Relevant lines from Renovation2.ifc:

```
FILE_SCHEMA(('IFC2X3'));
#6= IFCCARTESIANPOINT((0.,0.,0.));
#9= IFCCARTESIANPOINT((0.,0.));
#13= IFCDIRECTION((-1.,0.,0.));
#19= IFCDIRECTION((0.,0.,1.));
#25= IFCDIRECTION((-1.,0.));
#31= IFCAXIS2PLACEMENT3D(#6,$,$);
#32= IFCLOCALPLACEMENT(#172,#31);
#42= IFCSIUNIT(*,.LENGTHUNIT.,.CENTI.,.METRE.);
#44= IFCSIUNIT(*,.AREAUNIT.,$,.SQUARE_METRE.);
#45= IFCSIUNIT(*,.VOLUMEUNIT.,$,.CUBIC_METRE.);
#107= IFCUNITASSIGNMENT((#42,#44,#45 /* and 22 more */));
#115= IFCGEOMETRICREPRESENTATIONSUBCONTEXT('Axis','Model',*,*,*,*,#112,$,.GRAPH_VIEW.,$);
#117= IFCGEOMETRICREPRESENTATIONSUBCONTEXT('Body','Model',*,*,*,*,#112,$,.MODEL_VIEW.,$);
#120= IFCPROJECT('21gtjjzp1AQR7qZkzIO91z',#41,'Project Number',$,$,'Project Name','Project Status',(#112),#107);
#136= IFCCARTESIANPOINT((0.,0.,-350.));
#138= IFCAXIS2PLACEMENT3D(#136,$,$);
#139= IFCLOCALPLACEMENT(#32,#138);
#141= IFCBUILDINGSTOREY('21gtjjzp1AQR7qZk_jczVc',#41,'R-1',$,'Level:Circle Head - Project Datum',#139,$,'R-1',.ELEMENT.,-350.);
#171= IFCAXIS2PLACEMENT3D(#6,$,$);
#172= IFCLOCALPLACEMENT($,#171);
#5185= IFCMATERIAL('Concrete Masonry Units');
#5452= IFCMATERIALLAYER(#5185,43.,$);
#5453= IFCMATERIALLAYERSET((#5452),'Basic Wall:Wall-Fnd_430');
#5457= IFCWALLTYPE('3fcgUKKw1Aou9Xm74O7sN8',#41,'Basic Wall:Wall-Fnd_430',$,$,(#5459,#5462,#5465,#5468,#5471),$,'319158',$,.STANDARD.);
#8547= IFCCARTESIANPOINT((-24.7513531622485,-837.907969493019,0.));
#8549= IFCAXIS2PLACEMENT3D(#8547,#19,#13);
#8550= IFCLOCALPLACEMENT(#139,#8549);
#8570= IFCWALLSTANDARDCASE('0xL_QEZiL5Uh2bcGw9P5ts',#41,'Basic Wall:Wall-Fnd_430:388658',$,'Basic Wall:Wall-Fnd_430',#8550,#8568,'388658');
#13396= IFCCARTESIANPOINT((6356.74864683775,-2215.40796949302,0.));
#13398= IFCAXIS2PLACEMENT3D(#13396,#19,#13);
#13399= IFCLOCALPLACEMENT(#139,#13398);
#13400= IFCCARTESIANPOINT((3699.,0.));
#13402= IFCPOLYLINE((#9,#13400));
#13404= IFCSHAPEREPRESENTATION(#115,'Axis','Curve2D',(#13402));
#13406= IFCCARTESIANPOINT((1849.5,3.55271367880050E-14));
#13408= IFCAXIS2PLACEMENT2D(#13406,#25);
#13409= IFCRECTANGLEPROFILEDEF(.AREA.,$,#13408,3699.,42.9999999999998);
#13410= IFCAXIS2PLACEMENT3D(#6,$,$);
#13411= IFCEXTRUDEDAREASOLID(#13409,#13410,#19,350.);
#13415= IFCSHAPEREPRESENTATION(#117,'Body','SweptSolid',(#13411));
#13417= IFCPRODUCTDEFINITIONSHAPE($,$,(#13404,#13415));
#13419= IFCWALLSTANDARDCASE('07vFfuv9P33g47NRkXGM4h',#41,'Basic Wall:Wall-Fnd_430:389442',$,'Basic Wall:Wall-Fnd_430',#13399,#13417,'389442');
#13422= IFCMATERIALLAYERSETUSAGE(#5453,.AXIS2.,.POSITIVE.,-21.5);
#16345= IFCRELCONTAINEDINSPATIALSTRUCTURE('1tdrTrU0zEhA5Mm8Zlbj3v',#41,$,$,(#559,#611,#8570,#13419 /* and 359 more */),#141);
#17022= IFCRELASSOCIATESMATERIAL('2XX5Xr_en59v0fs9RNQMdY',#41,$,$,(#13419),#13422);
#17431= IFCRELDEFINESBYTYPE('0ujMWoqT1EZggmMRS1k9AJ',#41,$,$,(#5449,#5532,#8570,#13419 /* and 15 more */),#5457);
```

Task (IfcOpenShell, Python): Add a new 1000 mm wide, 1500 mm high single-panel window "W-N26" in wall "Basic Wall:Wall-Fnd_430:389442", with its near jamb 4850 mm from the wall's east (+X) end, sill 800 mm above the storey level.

```python
import numpy as np
import ifcopenshell
import ifcopenshell.api.feature
import ifcopenshell.api.geometry
import ifcopenshell.api.root
import ifcopenshell.api.spatial
import ifcopenshell.api.type
import ifcopenshell.geom
import ifcopenshell.util.element
import ifcopenshell.util.placement
import ifcopenshell.util.representation
import ifcopenshell.util.shape
import ifcopenshell.util.unit

model = ifcopenshell.open("Renovation2.ifc")
unit_scale = ifcopenshell.util.unit.calculate_unit_scale(model)
settings = ifcopenshell.geom.settings()


def volume(element):
    """Net volume in cubic metres, openings subtracted."""
    shape = ifcopenshell.geom.create_shape(settings, element)
    return ifcopenshell.util.shape.get_volume(shape.geometry)


wall = model.by_guid("07vFfuv9P33g47NRkXGM4h")
storey = ifcopenshell.util.element.get_container(wall, ifc_class="IfcBuildingStorey")
context = ifcopenshell.util.representation.get_context(model, "Model", "Body", "MODEL_VIEW")
before = volume(wall)

width, height, from_end, sill = 1, 1.5, 4.85, 0.8  # metres

# The wall runs along its own X axis, and the end named is its -X end.
wall_shape = ifcopenshell.geom.create_shape(settings, wall)
x, y, z = ifcopenshell.util.shape.get_vertices(wall_shape.geometry).T
start = x.min() + from_end
face, thickness = float(y.min()), float(y.max() - y.min())
wall_matrix = ifcopenshell.util.placement.get_local_placement(wall.ObjectPlacement)
level = ifcopenshell.util.placement.get_local_placement(storey.ObjectPlacement)[2, 3]


def in_wall(x, y):
    """Placement at x, y metres in the wall's axes, at sill height."""
    matrix = wall_matrix.copy()
    matrix[:, 3] = wall_matrix @ np.array([x / unit_scale, y / unit_scale, 0.0, 1.0])
    matrix[2, 3] = level + sill / unit_scale
    return matrix


# Opening: a box that overshoots both wall faces by 50 mm.
opening = ifcopenshell.api.root.create_entity(model, ifc_class="IfcOpeningElement")
box = ifcopenshell.api.geometry.add_wall_representation(
    model, context=context, length=width, height=height, thickness=thickness + 0.1
)
ifcopenshell.api.geometry.assign_representation(model, product=opening, representation=box)
ifcopenshell.api.geometry.edit_object_placement(model, product=opening, matrix=in_wall(start, face - 0.05), is_si=False)
ifcopenshell.api.feature.add_feature(model, feature=opening, element=wall)

window = ifcopenshell.api.root.create_entity(model, ifc_class="IfcWindow", name="W-N26")
window.OverallWidth, window.OverallHeight = width / unit_scale, height / unit_scale
body = ifcopenshell.api.geometry.add_window_representation(
    model,
    context=context,
    overall_width=window.OverallWidth,
    overall_height=window.OverallHeight,
    partition_type="SINGLE_PANEL",
)
ifcopenshell.api.geometry.assign_representation(model, product=window, representation=body)
ifcopenshell.api.spatial.assign_container(model, products=[window], relating_structure=storey)
fills = ifcopenshell.api.feature.add_filling(model, opening=opening, element=window)
fills.OwnerHistory = window.OwnerHistory  # required in IFC2X3

# IFC2X3 keeps the operation on the window style.
style = ifcopenshell.api.root.create_entity(model, ifc_class="IfcWindowStyle", name="W-N26")
style.OperationType, style.ConstructionType = "SINGLE_PANEL", "NOTDEFINED"
style.ParameterTakesPrecedence = style.Sizeable = False
ifcopenshell.api.type.assign_type(model, related_objects=[window], relating_type=style)

# Centre the window in the wall's thickness.
ifcopenshell.api.geometry.edit_object_placement(model, product=window, matrix=in_wall(start, face), is_si=False)
window_shape = ifcopenshell.geom.create_shape(settings, window)
depth = ifcopenshell.util.shape.get_vertices(window_shape.geometry)[:, 1]
offset = face + thickness / 2 - (depth.min() + depth.max()) / 2
ifcopenshell.api.geometry.edit_object_placement(model, product=window, matrix=in_wall(start, offset), is_si=False)

after = volume(wall)

print(f"wall volume {before:.3f} -> {after:.3f} m3")

model.write("Renovation2_updated.ifc")
```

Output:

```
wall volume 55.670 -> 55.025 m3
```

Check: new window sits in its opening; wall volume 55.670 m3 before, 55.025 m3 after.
